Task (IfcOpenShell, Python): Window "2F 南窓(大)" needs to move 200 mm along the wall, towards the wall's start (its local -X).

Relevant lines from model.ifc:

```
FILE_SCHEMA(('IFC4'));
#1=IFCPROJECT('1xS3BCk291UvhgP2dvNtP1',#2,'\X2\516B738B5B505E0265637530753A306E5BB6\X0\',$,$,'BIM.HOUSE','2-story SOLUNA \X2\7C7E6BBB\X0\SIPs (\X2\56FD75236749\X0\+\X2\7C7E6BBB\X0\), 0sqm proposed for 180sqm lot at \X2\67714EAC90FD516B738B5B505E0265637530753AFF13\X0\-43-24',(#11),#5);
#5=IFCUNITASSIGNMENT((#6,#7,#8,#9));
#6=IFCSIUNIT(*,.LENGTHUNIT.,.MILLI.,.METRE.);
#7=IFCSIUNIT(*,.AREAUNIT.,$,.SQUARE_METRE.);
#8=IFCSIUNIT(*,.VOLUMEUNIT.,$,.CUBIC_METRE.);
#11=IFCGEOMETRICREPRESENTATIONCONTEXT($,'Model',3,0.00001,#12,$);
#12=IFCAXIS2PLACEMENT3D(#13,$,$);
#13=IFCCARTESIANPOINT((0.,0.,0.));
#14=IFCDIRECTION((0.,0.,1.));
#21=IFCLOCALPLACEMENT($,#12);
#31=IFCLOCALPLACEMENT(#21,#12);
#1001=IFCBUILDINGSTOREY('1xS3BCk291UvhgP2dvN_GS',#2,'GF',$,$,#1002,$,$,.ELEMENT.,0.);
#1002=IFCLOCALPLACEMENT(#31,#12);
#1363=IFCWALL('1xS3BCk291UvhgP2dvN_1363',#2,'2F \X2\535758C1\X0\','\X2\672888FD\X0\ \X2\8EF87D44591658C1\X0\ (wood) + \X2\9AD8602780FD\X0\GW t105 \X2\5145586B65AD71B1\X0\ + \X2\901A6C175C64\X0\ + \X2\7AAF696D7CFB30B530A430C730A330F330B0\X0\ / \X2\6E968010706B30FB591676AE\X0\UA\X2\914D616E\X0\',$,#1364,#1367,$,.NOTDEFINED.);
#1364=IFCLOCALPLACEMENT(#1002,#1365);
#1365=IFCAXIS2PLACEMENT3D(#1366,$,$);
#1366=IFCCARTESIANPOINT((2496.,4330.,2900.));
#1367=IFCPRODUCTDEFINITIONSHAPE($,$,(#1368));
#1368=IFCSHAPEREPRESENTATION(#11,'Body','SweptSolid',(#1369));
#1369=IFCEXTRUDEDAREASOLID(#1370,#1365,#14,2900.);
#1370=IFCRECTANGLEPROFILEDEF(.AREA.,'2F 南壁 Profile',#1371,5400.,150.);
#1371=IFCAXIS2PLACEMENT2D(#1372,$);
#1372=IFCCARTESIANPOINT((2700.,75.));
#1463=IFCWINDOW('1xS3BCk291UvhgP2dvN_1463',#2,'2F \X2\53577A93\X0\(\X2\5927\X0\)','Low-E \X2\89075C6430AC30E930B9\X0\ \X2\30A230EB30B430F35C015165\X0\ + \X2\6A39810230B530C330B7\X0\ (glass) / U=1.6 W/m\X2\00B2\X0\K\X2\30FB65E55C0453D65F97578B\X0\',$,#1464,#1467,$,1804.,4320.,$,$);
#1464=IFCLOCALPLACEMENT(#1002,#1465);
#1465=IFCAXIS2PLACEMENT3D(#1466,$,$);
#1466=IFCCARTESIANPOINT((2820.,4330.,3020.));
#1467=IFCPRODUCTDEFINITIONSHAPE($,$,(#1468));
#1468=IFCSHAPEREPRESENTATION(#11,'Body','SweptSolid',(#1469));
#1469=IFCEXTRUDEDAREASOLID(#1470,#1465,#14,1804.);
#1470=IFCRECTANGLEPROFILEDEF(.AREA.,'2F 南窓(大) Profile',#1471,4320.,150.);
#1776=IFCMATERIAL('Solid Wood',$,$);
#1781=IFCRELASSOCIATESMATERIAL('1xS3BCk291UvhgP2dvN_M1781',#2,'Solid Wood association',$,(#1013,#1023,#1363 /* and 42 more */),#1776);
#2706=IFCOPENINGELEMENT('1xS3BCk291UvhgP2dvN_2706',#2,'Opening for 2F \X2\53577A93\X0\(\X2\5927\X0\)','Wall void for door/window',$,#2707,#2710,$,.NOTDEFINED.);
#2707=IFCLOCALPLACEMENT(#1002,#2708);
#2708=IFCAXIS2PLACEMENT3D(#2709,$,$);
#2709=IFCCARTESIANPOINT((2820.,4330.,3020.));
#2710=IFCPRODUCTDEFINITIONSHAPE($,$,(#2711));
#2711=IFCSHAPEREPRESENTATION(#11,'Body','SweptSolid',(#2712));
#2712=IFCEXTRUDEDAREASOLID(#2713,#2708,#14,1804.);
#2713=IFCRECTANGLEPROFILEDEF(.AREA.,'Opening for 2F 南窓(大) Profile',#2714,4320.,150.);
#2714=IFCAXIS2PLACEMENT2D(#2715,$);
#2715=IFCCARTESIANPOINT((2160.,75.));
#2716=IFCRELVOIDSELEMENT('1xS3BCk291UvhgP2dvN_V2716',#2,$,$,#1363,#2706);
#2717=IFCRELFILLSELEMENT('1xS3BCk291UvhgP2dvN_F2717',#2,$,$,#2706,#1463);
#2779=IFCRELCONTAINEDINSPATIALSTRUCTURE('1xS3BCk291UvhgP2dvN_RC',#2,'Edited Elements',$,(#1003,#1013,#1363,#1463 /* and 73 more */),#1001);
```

```python
import ifcopenshell
import ifcopenshell.api.geometry
import ifcopenshell.util.placement
import ifcopenshell.util.unit

model = ifcopenshell.open("model.ifc")
unit_scale = ifcopenshell.util.unit.calculate_unit_scale(model)

window = model.by_guid("1xS3BCk291UvhgP2dvN_1463")
opening = window.FillsVoids[0].RelatingOpeningElement
wall = opening.VoidsElements[0].RelatingBuildingElement

wall_matrix = ifcopenshell.util.placement.get_local_placement(wall.ObjectPlacement)
shift = wall_matrix[:3, 0] * -0.2 / unit_scale
before = ifcopenshell.util.placement.get_local_placement(window.ObjectPlacement)[:3, 3].copy()

# The window is not placed relative to its opening, so move both.
for product in (opening, window):
    matrix = ifcopenshell.util.placement.get_local_placement(product.ObjectPlacement)
    matrix[:3, 3] += shift
    ifcopenshell.api.geometry.edit_object_placement(model, product=product, matrix=matrix, is_si=False)

after = ifcopenshell.util.placement.get_local_placement(window.ObjectPlacement)[:3, 3]
print("window moved by", (after - before).round(3) + 0.0)

model.write("model-out.ifc")
```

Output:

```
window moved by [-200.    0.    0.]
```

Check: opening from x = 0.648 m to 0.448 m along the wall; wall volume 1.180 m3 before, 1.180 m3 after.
